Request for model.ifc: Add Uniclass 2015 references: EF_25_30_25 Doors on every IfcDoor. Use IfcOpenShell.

First a look at what the model holds.

```python
import ifcopenshell

model = ifcopenshell.open("model.ifc")
print(model.schema)
print("classifications:", [c.Name for c in model.by_type("IfcClassification")])
for ifc_class in ("IfcDoor", "IfcRoof", "IfcStair", "IfcWall", "IfcWindow"):
    print(ifc_class, len(model.by_type(ifc_class)))
```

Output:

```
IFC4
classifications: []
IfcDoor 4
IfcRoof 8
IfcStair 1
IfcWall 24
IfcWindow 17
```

```python
import ifcopenshell
import ifcopenshell.api.classification

model = ifcopenshell.open("model.ifc")

system = ifcopenshell.api.classification.add_classification(model, classification="Uniclass 2015")

codes = {
    "IfcDoor": ("EF_25_30_25", "Doors"),
}
for ifc_class, (code, name) in codes.items():
    products = model.by_type(ifc_class)
    ifcopenshell.api.classification.add_reference(
        model, products=products, classification=system, identification=code, name=name
    )
    print(code, len(products))

model.write("model_rev.ifc")
```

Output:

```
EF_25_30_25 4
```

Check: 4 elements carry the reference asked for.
